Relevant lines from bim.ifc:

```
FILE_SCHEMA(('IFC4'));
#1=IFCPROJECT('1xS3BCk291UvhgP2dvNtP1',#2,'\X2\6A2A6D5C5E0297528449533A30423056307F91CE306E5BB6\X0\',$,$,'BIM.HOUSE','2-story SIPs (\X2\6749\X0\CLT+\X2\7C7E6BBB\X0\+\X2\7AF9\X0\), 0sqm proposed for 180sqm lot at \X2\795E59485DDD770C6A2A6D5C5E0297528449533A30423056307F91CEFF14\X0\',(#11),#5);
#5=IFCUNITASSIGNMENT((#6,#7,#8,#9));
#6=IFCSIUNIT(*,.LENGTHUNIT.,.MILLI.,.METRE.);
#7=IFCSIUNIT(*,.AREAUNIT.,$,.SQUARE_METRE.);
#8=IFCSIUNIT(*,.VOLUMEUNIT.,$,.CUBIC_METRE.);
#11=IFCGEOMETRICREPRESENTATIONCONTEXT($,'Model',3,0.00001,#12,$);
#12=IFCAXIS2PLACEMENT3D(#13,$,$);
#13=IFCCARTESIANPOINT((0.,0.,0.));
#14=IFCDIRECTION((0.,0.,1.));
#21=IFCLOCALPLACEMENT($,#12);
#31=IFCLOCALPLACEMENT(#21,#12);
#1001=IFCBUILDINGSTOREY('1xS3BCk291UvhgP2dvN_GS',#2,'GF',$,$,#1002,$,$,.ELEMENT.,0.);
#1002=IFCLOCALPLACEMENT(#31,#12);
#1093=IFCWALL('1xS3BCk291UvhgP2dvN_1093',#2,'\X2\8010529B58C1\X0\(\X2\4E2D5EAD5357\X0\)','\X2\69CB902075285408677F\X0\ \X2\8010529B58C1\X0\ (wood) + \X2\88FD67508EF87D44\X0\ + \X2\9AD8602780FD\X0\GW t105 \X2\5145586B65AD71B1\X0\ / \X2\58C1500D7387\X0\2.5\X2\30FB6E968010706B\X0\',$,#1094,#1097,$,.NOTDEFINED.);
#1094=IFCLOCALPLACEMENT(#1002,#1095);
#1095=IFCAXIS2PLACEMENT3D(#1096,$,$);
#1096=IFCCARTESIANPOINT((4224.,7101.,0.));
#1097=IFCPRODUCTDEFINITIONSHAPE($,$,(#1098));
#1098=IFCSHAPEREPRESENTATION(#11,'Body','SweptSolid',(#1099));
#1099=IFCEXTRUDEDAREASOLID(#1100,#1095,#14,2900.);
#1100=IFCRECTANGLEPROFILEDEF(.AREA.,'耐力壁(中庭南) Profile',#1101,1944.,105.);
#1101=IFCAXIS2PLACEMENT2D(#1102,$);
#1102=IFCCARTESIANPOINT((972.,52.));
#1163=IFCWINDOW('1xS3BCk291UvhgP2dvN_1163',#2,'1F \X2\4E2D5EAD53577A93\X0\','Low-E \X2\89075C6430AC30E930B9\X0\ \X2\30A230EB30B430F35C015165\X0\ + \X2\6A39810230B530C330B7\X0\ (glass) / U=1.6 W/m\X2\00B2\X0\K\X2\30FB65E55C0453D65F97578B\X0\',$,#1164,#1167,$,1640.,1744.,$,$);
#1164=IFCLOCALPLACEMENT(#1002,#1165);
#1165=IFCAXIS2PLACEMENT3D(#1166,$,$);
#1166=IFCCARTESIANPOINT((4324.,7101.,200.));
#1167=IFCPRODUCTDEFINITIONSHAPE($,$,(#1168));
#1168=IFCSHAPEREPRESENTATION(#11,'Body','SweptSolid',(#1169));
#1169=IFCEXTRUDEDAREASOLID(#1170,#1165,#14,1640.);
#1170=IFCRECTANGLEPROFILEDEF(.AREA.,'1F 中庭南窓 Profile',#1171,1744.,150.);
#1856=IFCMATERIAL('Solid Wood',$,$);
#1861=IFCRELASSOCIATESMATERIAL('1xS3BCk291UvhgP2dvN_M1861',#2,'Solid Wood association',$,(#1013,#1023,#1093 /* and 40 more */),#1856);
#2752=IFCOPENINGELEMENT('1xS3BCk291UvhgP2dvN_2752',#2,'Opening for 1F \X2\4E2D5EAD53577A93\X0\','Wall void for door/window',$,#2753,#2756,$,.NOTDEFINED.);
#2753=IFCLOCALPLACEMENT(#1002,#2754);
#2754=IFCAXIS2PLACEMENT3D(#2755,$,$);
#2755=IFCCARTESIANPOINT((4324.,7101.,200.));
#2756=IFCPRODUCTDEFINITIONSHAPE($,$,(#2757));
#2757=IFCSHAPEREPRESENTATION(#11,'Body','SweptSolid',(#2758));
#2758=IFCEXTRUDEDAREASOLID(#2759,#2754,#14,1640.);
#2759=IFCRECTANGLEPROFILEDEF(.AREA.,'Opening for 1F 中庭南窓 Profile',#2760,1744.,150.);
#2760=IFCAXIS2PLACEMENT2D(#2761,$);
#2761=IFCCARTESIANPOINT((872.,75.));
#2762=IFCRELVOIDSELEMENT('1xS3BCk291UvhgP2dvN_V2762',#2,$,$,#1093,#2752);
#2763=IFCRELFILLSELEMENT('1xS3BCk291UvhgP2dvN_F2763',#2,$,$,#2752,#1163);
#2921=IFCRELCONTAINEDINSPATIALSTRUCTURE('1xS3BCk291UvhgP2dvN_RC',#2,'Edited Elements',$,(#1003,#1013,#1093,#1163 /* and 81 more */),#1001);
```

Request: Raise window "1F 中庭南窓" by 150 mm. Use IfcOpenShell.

```python
import numpy as np
import ifcopenshell
import ifcopenshell.api.geometry
import ifcopenshell.util.placement
import ifcopenshell.util.unit

model = ifcopenshell.open("bim.ifc")
unit_scale = ifcopenshell.util.unit.calculate_unit_scale(model)

window = model.by_id(1163)
opening = window.FillsVoids[0].RelatingOpeningElement
dz = 0.15 / unit_scale

shift = np.array([0.0, 0.0, dz])
# The window is not placed relative to its opening, so move both.
for product in (opening, window):
    matrix = ifcopenshell.util.placement.get_local_placement(product.ObjectPlacement)
    matrix[:3, 3] += shift
    ifcopenshell.api.geometry.edit_object_placement(model, product=product, matrix=matrix, is_si=False)

print(f"moved by {dz * unit_scale:+.3f} m")

model.write("bim_rev.ifc")
```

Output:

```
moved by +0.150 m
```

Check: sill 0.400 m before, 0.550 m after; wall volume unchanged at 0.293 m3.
